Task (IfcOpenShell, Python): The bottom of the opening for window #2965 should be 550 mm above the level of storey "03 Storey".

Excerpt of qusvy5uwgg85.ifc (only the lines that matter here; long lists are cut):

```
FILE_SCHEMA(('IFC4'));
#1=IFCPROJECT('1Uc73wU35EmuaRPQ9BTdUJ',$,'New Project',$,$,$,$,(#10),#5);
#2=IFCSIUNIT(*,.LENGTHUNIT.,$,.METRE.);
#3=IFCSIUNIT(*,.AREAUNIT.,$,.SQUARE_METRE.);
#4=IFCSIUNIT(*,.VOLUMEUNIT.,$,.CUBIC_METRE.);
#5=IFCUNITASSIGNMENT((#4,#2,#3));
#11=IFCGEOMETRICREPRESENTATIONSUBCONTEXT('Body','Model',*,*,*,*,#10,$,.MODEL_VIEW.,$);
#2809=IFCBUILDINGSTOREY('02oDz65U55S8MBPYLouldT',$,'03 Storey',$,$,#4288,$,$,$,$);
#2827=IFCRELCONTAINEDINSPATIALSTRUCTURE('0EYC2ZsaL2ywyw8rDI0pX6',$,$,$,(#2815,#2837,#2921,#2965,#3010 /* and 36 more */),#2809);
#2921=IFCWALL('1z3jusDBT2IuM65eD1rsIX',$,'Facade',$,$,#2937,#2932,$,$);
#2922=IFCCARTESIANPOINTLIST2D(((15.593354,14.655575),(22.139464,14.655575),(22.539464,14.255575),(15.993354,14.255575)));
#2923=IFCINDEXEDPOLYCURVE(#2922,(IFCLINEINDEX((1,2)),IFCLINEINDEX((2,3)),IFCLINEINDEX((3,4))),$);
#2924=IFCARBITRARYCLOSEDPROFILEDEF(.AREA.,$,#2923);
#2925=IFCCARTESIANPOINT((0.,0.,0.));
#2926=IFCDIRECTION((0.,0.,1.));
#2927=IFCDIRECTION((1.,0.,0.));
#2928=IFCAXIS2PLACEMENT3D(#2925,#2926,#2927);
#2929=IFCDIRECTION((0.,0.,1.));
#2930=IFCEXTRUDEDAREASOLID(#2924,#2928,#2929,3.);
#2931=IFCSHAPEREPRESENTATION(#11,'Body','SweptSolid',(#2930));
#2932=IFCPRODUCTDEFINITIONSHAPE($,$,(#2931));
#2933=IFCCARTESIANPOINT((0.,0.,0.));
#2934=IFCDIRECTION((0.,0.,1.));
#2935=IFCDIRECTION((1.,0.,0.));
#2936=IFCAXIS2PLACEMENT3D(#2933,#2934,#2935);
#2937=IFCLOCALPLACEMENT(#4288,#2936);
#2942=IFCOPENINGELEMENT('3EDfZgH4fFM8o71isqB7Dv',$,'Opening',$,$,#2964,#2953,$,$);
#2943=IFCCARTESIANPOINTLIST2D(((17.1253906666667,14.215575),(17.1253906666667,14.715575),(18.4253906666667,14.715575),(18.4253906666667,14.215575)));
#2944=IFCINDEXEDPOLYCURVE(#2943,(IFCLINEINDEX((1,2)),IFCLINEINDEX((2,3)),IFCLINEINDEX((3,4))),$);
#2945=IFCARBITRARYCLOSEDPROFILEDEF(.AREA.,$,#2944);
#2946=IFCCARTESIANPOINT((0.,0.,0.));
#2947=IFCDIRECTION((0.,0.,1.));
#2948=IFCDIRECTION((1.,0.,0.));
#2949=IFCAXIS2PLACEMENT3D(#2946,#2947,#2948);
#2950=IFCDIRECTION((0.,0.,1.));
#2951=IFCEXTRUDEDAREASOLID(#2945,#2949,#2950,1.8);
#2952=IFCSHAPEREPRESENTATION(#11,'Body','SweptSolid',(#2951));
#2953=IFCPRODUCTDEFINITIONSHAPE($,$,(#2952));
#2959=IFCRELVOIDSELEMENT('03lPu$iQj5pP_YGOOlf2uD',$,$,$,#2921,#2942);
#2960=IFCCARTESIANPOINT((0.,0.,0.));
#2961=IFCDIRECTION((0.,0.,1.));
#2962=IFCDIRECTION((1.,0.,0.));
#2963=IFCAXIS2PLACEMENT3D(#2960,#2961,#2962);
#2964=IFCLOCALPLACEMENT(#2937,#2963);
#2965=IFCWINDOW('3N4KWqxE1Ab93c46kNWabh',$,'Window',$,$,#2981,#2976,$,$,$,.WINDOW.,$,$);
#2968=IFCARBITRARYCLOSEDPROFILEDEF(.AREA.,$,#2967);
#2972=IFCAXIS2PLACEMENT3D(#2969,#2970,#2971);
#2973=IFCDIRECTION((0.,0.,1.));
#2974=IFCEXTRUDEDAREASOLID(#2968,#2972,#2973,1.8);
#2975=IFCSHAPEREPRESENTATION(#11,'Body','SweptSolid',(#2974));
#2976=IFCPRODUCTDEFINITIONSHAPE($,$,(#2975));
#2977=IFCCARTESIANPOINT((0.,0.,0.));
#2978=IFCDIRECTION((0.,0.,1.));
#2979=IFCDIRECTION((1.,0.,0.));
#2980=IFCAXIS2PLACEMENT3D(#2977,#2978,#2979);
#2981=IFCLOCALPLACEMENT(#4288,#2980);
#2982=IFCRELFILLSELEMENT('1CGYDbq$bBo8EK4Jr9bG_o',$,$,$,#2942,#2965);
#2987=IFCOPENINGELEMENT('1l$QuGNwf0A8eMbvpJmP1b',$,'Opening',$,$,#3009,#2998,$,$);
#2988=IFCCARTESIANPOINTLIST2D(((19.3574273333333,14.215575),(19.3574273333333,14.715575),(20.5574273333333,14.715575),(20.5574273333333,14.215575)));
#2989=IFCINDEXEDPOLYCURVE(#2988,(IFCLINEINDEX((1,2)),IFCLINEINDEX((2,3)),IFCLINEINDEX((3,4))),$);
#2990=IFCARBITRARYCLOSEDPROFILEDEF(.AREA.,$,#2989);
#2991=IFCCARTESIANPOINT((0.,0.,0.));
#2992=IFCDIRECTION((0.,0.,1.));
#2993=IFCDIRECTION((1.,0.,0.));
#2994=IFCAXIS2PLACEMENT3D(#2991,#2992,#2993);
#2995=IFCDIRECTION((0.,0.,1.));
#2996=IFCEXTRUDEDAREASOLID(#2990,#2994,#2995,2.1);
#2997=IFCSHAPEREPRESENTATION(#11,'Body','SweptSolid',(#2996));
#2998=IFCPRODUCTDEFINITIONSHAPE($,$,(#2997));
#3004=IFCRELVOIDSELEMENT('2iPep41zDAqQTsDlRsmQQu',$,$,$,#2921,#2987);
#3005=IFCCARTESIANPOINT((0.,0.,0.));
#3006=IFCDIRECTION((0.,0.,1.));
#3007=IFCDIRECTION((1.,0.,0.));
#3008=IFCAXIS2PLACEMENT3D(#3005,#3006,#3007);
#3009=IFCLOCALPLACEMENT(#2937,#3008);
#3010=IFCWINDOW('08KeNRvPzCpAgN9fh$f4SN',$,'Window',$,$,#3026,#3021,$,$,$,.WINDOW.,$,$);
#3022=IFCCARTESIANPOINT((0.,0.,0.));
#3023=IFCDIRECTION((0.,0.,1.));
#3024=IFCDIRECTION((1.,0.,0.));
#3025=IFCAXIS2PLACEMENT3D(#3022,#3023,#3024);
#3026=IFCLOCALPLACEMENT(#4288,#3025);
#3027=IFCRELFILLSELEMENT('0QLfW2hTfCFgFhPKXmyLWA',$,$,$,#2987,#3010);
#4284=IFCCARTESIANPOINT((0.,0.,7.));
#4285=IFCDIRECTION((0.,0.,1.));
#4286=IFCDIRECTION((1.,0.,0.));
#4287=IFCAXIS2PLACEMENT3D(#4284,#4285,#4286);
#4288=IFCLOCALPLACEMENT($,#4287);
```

```python
import numpy as np
import ifcopenshell
import ifcopenshell.api.geometry
import ifcopenshell.geom
import ifcopenshell.util.element
import ifcopenshell.util.placement
import ifcopenshell.util.shape
import ifcopenshell.util.unit

model = ifcopenshell.open("qusvy5uwgg85.ifc")
unit_scale = ifcopenshell.util.unit.calculate_unit_scale(model)

window = model.by_id(2965)
opening = window.FillsVoids[0].RelatingOpeningElement
storey = ifcopenshell.util.element.get_container(window, ifc_class="IfcBuildingStorey")
level = ifcopenshell.util.placement.get_local_placement(storey.ObjectPlacement)[2, 3]

# The opening's origin need not be at the sill, so measure its lowest point.
shape = ifcopenshell.geom.create_shape(ifcopenshell.geom.settings(), opening)
bottom = ifcopenshell.util.shape.get_shape_bottom_elevation(shape, shape.geometry) / unit_scale
dz = level + 0.55 / unit_scale - bottom

shift = np.array([0.0, 0.0, dz])
# The window is not placed relative to its opening, so move both.
for product in (opening, window):
    matrix = ifcopenshell.util.placement.get_local_placement(product.ObjectPlacement)
    matrix[:3, 3] += shift
    ifcopenshell.api.geometry.edit_object_placement(model, product=product, matrix=matrix, is_si=False)

print(f"moved by {dz * unit_scale:+.3f} m")

model.write("qusvy5uwgg85_rev.ifc")
```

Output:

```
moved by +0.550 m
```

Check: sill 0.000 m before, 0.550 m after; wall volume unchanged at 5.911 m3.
